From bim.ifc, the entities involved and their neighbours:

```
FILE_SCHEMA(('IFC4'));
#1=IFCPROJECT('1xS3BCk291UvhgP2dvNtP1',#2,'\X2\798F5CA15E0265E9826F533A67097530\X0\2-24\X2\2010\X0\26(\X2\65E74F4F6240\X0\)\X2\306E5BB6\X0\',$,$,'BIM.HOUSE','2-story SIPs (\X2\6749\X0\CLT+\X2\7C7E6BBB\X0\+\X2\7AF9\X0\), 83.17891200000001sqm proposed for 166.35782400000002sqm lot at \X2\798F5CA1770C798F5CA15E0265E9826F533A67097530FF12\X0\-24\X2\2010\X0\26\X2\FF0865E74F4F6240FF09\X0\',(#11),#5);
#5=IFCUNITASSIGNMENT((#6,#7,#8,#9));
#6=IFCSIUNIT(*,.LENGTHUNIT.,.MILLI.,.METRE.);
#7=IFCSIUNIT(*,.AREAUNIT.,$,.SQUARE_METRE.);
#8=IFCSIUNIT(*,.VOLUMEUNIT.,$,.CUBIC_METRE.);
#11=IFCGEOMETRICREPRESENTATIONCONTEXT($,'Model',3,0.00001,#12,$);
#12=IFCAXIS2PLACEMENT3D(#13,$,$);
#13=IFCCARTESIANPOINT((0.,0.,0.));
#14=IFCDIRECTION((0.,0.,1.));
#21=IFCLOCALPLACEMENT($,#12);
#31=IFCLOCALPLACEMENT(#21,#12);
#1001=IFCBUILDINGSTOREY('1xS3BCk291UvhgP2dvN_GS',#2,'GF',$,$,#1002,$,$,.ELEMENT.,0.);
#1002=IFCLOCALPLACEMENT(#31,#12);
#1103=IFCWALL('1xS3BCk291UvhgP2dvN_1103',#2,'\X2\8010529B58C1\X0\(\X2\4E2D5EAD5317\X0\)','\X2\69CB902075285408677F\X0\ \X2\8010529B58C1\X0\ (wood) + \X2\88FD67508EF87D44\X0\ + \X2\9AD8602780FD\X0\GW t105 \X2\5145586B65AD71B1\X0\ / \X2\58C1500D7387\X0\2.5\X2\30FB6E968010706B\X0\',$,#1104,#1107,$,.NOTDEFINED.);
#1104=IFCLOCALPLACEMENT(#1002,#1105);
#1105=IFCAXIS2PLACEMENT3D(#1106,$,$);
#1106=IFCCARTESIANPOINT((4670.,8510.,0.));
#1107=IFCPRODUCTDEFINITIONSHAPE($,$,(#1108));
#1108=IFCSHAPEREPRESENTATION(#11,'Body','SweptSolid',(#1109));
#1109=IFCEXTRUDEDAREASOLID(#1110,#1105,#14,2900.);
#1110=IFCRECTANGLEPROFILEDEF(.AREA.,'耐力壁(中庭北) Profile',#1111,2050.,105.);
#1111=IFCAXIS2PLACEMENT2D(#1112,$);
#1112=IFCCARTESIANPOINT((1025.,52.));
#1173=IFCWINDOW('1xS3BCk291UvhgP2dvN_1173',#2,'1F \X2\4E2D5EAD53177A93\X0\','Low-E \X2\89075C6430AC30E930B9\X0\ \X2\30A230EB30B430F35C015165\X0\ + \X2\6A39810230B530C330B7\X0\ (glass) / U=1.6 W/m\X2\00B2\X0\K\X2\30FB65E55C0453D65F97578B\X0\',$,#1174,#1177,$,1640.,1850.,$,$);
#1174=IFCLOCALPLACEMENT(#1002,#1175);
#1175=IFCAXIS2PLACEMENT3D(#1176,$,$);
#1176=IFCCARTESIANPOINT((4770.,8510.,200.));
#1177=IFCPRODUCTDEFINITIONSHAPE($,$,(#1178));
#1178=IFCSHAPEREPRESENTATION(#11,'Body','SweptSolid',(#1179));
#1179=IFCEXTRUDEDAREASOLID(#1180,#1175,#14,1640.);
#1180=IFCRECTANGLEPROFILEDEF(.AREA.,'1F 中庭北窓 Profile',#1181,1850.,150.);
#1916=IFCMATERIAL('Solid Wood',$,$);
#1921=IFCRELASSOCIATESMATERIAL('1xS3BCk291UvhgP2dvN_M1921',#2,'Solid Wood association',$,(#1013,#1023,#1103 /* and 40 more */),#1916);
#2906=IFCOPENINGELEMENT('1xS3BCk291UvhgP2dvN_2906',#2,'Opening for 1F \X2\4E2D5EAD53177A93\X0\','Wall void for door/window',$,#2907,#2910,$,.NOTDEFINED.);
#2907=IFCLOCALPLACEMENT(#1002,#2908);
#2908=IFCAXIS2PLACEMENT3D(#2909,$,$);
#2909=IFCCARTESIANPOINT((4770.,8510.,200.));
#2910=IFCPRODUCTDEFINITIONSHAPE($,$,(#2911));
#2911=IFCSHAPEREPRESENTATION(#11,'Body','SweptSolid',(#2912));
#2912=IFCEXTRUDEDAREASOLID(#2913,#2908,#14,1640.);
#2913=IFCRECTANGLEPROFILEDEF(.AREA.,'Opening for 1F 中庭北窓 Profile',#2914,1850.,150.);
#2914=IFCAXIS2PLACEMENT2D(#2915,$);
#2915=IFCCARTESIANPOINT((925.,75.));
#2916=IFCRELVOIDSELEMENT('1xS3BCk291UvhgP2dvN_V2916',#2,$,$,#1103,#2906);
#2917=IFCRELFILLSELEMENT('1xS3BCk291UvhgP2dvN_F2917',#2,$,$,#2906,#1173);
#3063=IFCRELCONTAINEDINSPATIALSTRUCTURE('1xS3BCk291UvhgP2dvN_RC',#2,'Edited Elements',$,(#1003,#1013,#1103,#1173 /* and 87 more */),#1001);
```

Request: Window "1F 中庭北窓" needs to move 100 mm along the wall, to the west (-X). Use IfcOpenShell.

```python
import ifcopenshell
import ifcopenshell.api.geometry
import ifcopenshell.util.placement
import ifcopenshell.util.unit

model = ifcopenshell.open("bim.ifc")
unit_scale = ifcopenshell.util.unit.calculate_unit_scale(model)

window = model.by_guid("1xS3BCk291UvhgP2dvN_1173")
opening = window.FillsVoids[0].RelatingOpeningElement
wall = opening.VoidsElements[0].RelatingBuildingElement

wall_matrix = ifcopenshell.util.placement.get_local_placement(wall.ObjectPlacement)
shift = wall_matrix[:3, 0] * -0.1 / unit_scale
before = ifcopenshell.util.placement.get_local_placement(window.ObjectPlacement)[:3, 3].copy()

# The window is not placed relative to its opening, so move both.
for product in (opening, window):
    matrix = ifcopenshell.util.placement.get_local_placement(product.ObjectPlacement)
    matrix[:3, 3] += shift
    ifcopenshell.api.geometry.edit_object_placement(model, product=product, matrix=matrix, is_si=False)

after = ifcopenshell.util.placement.get_local_placement(window.ObjectPlacement)[:3, 3]
print("window moved by", (after - before).round(3) + 0.0)

model.write("bim_rev.ifc")
```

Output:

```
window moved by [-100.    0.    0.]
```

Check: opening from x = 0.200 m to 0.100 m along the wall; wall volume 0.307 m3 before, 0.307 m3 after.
